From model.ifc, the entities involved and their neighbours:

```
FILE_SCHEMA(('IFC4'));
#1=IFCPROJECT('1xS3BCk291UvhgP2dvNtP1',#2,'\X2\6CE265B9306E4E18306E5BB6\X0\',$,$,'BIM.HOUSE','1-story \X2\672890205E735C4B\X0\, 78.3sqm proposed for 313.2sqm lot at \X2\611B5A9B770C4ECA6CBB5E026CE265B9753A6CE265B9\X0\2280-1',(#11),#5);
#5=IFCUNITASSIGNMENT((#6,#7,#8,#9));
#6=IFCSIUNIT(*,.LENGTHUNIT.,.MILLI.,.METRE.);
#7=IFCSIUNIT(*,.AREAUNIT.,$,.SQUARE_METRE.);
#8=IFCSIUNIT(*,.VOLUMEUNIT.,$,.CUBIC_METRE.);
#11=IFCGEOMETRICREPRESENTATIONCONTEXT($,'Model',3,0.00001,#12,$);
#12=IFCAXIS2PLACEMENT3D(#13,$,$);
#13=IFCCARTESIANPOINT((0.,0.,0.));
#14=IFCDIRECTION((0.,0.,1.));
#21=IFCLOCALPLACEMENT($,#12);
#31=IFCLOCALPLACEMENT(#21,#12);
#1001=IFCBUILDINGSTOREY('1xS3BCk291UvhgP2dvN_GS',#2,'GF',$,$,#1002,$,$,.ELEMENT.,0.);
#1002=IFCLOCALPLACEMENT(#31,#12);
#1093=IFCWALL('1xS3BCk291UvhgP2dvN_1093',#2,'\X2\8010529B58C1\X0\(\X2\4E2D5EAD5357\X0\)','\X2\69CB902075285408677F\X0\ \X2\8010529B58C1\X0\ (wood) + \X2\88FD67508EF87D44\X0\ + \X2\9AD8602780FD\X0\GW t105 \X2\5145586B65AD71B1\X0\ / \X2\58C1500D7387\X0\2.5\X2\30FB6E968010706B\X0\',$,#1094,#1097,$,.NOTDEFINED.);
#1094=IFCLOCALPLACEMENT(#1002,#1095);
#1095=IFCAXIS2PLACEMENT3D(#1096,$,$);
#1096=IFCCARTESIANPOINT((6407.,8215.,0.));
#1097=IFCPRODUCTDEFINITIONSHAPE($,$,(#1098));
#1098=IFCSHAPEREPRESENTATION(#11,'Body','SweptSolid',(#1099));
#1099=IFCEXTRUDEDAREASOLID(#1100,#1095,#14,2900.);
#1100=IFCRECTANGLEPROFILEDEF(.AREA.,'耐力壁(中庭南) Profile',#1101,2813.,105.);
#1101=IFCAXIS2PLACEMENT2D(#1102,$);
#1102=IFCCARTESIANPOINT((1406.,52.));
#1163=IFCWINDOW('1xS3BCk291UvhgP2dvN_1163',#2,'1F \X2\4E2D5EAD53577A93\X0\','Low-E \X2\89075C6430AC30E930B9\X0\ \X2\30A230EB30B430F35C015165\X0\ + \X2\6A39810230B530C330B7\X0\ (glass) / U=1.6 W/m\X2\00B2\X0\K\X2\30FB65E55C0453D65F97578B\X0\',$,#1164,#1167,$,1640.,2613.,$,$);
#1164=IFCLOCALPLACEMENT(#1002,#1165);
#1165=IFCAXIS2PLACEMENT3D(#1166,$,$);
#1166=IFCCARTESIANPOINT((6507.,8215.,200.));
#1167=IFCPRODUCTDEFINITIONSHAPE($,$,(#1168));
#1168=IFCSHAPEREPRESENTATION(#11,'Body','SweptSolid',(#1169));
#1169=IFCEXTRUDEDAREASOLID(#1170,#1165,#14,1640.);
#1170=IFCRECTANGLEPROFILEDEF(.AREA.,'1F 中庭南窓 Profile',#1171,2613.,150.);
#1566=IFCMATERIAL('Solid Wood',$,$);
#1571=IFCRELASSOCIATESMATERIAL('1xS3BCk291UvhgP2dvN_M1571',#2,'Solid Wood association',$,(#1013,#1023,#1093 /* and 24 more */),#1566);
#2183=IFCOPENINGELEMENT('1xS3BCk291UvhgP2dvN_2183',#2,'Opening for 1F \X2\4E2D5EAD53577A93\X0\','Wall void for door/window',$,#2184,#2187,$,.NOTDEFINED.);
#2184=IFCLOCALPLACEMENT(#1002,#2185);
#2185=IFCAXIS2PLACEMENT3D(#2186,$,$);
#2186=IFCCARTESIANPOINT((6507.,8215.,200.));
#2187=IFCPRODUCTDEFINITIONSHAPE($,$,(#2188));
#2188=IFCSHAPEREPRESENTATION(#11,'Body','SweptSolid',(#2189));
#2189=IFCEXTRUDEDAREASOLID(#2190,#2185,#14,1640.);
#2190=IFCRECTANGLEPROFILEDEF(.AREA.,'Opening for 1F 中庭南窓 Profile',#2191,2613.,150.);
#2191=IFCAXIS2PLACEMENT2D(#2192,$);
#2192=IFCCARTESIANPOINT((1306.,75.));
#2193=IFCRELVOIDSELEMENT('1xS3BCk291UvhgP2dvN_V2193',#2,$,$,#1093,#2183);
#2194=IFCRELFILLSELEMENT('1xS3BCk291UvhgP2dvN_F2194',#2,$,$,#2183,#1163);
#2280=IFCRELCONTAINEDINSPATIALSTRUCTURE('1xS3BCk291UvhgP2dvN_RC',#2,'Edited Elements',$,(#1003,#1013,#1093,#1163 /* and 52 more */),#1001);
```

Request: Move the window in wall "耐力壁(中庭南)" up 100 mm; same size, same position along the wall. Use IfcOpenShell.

```python
import numpy as np
import ifcopenshell
import ifcopenshell.api.geometry
import ifcopenshell.util.placement
import ifcopenshell.util.unit

model = ifcopenshell.open("model.ifc")
unit_scale = ifcopenshell.util.unit.calculate_unit_scale(model)

window = model.by_id(1163)
opening = window.FillsVoids[0].RelatingOpeningElement
dz = 0.1 / unit_scale

shift = np.array([0.0, 0.0, dz])
# The window is not placed relative to its opening, so move both.
for product in (opening, window):
    matrix = ifcopenshell.util.placement.get_local_placement(product.ObjectPlacement)
    matrix[:3, 3] += shift
    ifcopenshell.api.geometry.edit_object_placement(model, product=product, matrix=matrix, is_si=False)

print(f"moved by {dz * unit_scale:+.3f} m")

model.write("model_updated.ifc")
```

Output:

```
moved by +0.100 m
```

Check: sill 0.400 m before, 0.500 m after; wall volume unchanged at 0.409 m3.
